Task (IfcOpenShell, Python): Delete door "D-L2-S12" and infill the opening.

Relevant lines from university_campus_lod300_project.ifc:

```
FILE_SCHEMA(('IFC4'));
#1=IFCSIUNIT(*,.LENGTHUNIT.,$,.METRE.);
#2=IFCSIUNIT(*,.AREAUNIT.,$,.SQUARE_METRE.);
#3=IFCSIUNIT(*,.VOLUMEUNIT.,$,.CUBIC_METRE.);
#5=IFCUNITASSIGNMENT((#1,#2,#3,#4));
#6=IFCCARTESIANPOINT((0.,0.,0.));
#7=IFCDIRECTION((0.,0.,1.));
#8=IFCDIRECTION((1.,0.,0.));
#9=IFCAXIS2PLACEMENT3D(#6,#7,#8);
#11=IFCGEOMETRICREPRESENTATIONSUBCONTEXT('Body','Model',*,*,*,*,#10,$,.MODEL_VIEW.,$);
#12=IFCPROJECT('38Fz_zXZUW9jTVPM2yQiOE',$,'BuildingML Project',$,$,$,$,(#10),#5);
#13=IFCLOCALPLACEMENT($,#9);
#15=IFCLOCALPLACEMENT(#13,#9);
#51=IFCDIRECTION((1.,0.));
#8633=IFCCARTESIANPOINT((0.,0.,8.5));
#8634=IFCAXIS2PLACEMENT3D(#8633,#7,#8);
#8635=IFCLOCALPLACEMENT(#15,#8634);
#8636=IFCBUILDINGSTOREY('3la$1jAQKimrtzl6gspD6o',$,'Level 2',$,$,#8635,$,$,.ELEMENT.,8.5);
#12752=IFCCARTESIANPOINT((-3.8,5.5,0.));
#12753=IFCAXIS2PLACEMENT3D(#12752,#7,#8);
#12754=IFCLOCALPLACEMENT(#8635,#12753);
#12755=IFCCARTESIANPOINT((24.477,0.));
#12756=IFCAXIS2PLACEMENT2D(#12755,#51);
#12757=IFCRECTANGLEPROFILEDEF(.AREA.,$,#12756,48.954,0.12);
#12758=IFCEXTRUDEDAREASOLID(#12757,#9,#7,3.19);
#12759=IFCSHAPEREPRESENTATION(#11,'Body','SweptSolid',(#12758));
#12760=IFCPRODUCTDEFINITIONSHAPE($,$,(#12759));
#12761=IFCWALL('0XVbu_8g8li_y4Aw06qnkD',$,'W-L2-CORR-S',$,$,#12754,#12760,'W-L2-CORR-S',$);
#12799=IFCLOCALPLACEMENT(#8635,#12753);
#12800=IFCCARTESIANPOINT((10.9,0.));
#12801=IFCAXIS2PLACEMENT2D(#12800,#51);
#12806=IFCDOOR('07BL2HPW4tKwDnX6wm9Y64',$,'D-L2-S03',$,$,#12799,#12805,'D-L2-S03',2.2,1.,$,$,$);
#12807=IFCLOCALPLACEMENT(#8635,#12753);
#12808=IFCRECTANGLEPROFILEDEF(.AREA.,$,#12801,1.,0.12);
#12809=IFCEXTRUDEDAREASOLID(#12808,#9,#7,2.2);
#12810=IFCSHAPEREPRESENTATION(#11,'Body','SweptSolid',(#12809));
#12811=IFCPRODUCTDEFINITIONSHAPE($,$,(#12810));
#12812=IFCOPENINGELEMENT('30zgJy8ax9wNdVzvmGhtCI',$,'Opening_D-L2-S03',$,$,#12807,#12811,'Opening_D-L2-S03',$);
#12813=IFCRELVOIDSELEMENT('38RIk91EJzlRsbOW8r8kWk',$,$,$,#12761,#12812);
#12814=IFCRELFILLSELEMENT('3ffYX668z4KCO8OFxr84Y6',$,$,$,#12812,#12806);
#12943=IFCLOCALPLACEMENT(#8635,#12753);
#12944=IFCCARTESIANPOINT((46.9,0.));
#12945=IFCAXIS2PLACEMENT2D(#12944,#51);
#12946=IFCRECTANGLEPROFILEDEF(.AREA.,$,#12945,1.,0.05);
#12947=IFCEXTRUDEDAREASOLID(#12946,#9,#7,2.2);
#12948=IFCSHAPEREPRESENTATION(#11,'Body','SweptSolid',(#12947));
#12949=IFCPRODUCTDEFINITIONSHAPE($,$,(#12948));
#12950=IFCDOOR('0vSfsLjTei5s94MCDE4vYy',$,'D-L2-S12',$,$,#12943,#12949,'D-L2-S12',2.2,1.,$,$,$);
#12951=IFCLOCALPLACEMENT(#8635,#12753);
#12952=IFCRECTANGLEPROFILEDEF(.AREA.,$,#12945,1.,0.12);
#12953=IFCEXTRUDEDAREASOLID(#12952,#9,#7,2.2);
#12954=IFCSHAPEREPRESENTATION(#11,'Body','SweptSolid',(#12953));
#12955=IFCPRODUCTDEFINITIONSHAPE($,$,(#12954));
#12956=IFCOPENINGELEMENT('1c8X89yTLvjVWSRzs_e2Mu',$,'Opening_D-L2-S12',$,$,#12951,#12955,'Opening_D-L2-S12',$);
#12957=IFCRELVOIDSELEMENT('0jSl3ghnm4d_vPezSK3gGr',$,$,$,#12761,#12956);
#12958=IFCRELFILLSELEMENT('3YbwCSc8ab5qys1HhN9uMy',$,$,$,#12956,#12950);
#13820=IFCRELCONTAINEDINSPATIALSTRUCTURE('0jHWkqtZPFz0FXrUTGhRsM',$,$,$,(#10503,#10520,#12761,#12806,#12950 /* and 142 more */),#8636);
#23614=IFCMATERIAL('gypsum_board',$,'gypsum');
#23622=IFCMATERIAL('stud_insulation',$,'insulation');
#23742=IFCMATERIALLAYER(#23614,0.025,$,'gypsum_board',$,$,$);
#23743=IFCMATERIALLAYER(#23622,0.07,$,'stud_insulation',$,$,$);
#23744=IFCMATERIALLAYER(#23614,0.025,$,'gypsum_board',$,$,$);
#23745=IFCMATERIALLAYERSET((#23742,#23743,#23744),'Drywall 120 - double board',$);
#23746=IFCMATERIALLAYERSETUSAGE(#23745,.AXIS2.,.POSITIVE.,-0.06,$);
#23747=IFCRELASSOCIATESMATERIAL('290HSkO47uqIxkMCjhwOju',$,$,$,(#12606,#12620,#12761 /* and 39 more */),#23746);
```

```python
import ifcopenshell
import ifcopenshell.api.feature
import ifcopenshell.api.root
import ifcopenshell.geom
import ifcopenshell.util.shape

model = ifcopenshell.open("university_campus_lod300_project.ifc")
settings = ifcopenshell.geom.settings()


def volume(element):
    """Net volume in cubic metres, openings subtracted."""
    shape = ifcopenshell.geom.create_shape(settings, element)
    return ifcopenshell.util.shape.get_volume(shape.geometry)


door = model.by_id(12950)
opening = door.FillsVoids[0].RelatingOpeningElement
wall = opening.VoidsElements[0].RelatingBuildingElement
before = volume(wall)

ifcopenshell.api.root.remove_product(model, product=door)
ifcopenshell.api.feature.remove_feature(model, feature=opening)

after = volume(wall)

print(f"wall volume {before:.3f} -> {after:.3f} m3")

model.write("university_campus_lod300_project_rev.ifc")
```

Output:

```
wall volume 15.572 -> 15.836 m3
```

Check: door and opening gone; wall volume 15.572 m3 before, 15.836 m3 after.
